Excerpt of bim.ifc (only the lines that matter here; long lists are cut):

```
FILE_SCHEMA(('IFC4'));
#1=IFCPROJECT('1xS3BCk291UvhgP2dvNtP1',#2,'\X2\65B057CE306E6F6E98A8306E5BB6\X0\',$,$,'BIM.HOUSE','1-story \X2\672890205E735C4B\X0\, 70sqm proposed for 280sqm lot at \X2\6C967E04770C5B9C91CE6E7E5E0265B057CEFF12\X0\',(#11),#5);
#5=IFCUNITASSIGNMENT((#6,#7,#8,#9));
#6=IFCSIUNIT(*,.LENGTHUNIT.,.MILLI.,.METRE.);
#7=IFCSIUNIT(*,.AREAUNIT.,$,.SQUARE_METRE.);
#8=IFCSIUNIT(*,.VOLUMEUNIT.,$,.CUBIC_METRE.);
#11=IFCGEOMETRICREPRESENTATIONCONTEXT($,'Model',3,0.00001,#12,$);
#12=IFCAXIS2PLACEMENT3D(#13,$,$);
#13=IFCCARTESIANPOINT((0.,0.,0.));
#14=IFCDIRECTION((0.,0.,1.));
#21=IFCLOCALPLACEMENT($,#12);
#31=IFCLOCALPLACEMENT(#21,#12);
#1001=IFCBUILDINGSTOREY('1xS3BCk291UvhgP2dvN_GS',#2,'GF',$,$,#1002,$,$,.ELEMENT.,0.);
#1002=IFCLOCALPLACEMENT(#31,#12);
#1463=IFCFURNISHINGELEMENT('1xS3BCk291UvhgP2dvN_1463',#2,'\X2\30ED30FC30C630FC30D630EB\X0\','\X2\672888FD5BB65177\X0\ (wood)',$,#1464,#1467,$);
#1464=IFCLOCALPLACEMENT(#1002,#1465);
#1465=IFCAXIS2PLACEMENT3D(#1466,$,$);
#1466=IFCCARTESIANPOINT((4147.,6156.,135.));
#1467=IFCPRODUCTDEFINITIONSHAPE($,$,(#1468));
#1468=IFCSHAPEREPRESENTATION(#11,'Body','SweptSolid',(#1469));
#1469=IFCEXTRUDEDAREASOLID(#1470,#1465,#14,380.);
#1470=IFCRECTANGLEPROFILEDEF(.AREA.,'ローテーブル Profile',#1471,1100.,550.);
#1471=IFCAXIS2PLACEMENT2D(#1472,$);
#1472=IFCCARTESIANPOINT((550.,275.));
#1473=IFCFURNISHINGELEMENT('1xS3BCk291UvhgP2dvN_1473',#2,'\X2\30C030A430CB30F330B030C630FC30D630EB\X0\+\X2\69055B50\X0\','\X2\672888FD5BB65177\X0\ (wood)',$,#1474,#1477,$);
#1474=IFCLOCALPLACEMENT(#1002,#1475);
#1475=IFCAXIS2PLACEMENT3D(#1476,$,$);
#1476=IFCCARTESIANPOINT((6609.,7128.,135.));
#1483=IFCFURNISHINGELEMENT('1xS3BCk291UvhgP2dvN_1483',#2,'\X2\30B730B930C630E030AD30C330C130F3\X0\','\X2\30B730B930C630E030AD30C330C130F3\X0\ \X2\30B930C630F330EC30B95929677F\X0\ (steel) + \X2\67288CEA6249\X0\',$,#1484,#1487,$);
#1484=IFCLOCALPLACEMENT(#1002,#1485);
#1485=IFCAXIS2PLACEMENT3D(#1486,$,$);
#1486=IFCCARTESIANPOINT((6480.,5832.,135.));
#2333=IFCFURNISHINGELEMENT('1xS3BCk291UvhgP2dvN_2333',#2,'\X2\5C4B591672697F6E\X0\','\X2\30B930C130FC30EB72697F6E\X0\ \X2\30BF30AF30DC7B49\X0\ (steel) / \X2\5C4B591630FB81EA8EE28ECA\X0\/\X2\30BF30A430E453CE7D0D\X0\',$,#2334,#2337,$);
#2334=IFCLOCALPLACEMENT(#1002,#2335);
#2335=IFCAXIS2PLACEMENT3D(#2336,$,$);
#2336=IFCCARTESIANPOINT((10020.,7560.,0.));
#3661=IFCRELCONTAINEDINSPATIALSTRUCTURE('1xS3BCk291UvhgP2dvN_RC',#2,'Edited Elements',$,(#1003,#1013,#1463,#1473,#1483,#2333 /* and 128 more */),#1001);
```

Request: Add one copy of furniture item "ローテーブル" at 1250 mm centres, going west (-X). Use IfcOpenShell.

```python
import numpy as np
import ifcopenshell
import ifcopenshell.api.geometry
import ifcopenshell.api.root
import ifcopenshell.util.element
import ifcopenshell.util.placement

model = ifcopenshell.open("bim.ifc")


def reuse_history(source, copy):
    """copy_class also copies each property set's owner history, people and application; keep the originals."""
    for rel in copy.IsDefinedBy:
        if rel.is_a("IfcRelDefinesByProperties") and (history := rel.RelatingPropertyDefinition.OwnerHistory):
            rel.RelatingPropertyDefinition.OwnerHistory = source.OwnerHistory
            ifcopenshell.util.element.remove_deep2(model, history)


source = model.by_id(1463)
base = ifcopenshell.util.placement.get_local_placement(source.ObjectPlacement)
step = np.array([-1.0, 0.0, 0.0]) * 1250.0

for i in range(1, 2):
    copy = ifcopenshell.api.root.copy_class(model, product=source)
    copy.Representation = ifcopenshell.util.element.copy_deep(
        model, source.Representation, exclude=["IfcGeometricRepresentationContext", "IfcRepresentationMap"]
    )
    reuse_history(source, copy)
    matrix = base.copy()
    matrix[:3, 3] += i * step
    print("added at", matrix[:3, 3].round(3) + 0.0)
    ifcopenshell.api.geometry.edit_object_placement(model, product=copy, matrix=matrix, is_si=False)

model.write("bim_edited.ifc")
```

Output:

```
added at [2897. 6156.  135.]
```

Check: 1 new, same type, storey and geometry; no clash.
